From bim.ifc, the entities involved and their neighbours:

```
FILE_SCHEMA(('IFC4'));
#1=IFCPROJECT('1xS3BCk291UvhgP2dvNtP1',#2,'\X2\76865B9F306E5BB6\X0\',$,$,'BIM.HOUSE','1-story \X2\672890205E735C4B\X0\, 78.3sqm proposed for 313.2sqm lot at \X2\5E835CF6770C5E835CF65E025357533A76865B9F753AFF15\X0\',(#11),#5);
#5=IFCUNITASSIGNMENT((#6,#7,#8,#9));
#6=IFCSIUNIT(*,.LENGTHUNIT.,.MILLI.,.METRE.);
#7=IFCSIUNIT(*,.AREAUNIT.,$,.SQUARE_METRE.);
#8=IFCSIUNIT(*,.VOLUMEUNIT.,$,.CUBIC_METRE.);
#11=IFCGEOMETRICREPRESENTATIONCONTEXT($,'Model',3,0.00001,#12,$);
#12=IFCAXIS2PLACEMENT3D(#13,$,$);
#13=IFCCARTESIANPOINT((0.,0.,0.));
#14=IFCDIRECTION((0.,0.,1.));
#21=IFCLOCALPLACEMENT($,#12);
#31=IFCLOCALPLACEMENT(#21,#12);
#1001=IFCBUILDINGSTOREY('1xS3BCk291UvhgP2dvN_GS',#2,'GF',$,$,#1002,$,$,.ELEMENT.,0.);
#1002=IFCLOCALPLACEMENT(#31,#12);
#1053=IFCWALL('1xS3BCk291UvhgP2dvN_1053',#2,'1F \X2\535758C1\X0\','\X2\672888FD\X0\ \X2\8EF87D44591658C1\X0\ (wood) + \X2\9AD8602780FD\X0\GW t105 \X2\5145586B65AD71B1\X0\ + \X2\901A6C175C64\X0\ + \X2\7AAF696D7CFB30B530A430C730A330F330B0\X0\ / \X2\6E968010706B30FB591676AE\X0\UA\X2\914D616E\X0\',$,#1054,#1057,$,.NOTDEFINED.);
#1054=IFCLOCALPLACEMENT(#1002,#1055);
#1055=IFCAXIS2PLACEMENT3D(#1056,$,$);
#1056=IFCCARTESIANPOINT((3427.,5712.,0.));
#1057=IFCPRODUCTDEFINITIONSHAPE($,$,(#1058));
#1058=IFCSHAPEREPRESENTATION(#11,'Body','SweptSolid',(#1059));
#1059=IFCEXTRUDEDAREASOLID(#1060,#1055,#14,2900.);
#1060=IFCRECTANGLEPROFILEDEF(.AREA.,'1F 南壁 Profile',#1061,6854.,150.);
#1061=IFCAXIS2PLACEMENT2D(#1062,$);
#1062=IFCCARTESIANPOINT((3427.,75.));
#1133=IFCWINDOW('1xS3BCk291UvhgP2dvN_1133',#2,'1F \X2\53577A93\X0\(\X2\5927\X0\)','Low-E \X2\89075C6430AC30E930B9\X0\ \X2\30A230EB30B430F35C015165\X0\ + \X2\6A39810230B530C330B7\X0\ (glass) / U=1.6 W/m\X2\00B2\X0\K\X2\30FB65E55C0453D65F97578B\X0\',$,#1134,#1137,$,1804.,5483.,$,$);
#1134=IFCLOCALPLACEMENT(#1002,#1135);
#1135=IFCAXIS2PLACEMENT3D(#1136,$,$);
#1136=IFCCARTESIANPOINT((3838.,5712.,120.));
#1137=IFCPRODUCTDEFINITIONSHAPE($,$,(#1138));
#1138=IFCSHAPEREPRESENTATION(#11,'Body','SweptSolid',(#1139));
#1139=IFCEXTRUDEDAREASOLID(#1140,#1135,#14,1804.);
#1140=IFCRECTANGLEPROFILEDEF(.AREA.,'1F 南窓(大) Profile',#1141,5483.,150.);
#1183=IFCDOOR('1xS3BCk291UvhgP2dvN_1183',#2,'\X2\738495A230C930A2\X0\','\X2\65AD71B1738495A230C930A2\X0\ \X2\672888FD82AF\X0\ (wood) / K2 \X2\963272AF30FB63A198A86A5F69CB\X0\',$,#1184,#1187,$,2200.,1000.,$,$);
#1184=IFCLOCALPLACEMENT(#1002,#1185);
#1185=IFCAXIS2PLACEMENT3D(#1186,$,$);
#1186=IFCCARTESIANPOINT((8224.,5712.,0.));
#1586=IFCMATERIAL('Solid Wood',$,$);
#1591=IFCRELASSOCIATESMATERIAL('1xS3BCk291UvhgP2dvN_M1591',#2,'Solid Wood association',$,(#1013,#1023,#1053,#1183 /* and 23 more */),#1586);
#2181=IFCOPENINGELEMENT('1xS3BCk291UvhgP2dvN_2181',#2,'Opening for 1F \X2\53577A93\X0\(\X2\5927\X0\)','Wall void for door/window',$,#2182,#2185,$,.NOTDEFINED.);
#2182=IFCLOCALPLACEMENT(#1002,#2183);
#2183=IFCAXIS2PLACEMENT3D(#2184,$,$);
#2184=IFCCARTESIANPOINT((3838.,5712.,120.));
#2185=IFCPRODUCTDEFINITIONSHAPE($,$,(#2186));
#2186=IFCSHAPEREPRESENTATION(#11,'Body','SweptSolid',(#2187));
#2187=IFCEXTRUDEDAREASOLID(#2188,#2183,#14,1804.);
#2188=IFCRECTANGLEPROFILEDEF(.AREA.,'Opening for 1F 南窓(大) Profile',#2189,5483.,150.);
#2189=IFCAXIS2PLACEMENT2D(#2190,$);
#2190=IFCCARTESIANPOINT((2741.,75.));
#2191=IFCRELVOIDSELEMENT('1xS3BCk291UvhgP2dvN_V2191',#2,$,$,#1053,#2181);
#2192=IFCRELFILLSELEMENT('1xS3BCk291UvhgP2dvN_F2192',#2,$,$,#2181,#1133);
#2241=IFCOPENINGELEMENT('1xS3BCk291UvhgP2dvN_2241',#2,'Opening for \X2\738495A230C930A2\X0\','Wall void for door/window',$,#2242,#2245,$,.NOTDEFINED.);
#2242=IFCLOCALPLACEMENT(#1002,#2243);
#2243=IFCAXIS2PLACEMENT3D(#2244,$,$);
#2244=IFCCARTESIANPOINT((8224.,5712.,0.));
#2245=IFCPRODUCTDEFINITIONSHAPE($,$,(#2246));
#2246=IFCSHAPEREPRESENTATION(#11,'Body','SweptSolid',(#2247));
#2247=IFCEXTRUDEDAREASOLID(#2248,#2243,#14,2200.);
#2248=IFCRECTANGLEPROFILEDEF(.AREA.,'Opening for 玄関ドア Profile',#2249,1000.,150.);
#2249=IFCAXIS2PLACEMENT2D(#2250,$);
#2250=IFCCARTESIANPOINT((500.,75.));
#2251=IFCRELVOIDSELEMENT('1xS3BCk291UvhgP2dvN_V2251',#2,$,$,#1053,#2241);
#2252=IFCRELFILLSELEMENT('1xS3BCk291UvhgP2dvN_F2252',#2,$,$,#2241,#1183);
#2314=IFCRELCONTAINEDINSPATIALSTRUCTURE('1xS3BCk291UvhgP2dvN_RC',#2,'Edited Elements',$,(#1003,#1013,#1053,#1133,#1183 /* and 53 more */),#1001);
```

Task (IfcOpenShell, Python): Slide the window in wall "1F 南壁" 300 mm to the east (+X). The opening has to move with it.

```python
import ifcopenshell
import ifcopenshell.api.geometry
import ifcopenshell.util.placement

model = ifcopenshell.open("bim.ifc")

window = model.by_guid("1xS3BCk291UvhgP2dvN_1133")
opening = window.FillsVoids[0].RelatingOpeningElement
wall = opening.VoidsElements[0].RelatingBuildingElement

wall_matrix = ifcopenshell.util.placement.get_local_placement(wall.ObjectPlacement)
shift = wall_matrix[:3, 0] * 300.0
before = ifcopenshell.util.placement.get_local_placement(window.ObjectPlacement)[:3, 3].copy()

# The window is not placed relative to its opening, so move both.
for product in (opening, window):
    matrix = ifcopenshell.util.placement.get_local_placement(product.ObjectPlacement)
    matrix[:3, 3] += shift
    ifcopenshell.api.geometry.edit_object_placement(model, product=product, matrix=matrix, is_si=False)

after = ifcopenshell.util.placement.get_local_placement(window.ObjectPlacement)[:3, 3]
print("window moved by", (after - before).round(3) + 0.0)

model.write("bim_v2.ifc")
```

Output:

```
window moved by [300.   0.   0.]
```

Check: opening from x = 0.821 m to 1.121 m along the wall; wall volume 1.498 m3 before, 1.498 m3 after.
